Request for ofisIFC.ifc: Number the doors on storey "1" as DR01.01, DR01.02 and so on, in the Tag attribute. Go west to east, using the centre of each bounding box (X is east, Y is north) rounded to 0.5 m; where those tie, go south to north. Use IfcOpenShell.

First a look at what the model holds.

```python
import ifcopenshell
import ifcopenshell.util.element
import ifcopenshell.util.placement

model = ifcopenshell.open("ofisIFC.ifc")
print(model.schema)
storey = next(s for s in model.by_type("IfcBuildingStorey") if s.Name == "1")
doors = [e for e in ifcopenshell.util.element.get_decomposition(storey) if e.is_a("IfcDoor")]
for e in sorted(doors, key=lambda e: e.id()):
    origin = ifcopenshell.util.placement.get_local_placement(e.ObjectPlacement)[:3, 3]
    print(e.id(), e.Tag, e.Name, origin.round(2) + 0.0, sep=" | ")
```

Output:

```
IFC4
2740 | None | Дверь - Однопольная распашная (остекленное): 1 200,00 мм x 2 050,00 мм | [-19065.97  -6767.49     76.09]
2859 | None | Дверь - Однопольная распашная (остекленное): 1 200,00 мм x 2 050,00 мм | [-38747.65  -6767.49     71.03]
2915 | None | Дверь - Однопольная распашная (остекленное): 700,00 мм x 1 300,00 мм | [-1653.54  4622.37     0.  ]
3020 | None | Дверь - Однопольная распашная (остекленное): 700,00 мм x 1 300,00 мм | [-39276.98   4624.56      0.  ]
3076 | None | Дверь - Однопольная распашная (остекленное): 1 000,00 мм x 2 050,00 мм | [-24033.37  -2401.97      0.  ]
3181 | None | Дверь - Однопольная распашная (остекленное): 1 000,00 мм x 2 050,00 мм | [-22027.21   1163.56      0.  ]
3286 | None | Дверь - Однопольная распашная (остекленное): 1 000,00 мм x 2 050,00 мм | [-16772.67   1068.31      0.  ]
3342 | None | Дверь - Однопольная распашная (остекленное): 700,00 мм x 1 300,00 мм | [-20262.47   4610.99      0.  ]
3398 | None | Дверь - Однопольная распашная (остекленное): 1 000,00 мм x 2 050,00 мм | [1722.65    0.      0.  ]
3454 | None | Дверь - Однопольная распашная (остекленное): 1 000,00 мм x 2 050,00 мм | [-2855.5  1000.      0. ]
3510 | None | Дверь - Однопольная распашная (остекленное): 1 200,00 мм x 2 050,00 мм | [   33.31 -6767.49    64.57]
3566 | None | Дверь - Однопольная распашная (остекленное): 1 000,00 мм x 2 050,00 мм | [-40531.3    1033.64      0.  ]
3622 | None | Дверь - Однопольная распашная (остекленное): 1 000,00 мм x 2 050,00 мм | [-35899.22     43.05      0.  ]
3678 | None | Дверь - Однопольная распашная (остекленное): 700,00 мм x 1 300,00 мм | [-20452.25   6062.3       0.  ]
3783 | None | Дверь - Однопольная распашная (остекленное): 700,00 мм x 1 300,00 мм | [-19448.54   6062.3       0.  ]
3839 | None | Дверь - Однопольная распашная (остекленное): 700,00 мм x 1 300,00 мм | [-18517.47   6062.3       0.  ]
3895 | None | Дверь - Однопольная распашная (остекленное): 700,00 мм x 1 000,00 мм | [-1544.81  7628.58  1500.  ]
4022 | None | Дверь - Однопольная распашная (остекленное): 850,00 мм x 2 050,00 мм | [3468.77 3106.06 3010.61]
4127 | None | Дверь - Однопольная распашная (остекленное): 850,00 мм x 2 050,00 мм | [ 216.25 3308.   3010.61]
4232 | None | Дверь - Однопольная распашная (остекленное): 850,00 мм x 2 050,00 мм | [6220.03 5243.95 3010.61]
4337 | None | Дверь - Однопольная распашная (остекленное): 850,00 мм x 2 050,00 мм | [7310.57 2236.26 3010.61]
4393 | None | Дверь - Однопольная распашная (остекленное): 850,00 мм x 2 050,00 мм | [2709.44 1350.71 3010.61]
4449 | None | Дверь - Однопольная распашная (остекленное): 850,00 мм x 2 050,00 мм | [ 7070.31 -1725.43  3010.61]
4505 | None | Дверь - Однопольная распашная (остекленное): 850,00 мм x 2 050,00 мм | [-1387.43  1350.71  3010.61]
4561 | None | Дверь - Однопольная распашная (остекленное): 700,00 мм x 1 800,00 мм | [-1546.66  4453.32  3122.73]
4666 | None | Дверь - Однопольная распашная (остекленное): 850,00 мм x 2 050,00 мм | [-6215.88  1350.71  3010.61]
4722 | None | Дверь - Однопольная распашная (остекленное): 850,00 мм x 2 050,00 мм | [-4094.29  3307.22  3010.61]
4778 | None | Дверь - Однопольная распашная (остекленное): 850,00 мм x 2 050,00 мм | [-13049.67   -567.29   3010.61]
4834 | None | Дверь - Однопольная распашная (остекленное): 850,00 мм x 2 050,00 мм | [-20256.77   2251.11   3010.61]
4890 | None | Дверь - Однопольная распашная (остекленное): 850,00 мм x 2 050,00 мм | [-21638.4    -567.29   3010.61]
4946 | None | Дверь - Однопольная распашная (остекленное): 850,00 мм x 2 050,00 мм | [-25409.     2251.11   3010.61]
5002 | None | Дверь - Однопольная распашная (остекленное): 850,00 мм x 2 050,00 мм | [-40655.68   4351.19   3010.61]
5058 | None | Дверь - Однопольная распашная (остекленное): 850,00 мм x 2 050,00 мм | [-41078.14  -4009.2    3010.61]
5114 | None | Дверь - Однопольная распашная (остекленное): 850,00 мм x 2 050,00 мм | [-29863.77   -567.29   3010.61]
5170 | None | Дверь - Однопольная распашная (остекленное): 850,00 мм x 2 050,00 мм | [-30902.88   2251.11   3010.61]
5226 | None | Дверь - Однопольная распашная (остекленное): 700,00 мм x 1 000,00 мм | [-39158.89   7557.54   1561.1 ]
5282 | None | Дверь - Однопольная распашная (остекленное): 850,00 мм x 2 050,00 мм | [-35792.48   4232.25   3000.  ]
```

```python
import ifcopenshell
import ifcopenshell.geom
import ifcopenshell.util.element
import ifcopenshell.util.shape

model = ifcopenshell.open("ofisIFC.ifc")
settings = ifcopenshell.geom.settings()
settings.set("use-world-coords", True)


def centre(element):
    shape = ifcopenshell.geom.create_shape(settings, element)
    return ifcopenshell.util.shape.get_bbox_centroid(shape.geometry)


storey = next(s for s in model.by_type("IfcBuildingStorey") if s.Name == "1")
doors = [e for e in ifcopenshell.util.element.get_decomposition(storey) if e.is_a("IfcDoor")]

# Insertion points can sit at a corner or the storey origin, so sort by the geometry (in metres).
centres = {e: centre(e) for e in doors}
doors.sort(key=lambda e: (round(centres[e][0] / 0.5), centres[e][1]))

for i, e in enumerate(doors, start=1):
    number = f"DR01.{i:02d}"
    e.Tag = number
    print(e.id(), number)

model.write("ofisIFC_edited.ifc")
```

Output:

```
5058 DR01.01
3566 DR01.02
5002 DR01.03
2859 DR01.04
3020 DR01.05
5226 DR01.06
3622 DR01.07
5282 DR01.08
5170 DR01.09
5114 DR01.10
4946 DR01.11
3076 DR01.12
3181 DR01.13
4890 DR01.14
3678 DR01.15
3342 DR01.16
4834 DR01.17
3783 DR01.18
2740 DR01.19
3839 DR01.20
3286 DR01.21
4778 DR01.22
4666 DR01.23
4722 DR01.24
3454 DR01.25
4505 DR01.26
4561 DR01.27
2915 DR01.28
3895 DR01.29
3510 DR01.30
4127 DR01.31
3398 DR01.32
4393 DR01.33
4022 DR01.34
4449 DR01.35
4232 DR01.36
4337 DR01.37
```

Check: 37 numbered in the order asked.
